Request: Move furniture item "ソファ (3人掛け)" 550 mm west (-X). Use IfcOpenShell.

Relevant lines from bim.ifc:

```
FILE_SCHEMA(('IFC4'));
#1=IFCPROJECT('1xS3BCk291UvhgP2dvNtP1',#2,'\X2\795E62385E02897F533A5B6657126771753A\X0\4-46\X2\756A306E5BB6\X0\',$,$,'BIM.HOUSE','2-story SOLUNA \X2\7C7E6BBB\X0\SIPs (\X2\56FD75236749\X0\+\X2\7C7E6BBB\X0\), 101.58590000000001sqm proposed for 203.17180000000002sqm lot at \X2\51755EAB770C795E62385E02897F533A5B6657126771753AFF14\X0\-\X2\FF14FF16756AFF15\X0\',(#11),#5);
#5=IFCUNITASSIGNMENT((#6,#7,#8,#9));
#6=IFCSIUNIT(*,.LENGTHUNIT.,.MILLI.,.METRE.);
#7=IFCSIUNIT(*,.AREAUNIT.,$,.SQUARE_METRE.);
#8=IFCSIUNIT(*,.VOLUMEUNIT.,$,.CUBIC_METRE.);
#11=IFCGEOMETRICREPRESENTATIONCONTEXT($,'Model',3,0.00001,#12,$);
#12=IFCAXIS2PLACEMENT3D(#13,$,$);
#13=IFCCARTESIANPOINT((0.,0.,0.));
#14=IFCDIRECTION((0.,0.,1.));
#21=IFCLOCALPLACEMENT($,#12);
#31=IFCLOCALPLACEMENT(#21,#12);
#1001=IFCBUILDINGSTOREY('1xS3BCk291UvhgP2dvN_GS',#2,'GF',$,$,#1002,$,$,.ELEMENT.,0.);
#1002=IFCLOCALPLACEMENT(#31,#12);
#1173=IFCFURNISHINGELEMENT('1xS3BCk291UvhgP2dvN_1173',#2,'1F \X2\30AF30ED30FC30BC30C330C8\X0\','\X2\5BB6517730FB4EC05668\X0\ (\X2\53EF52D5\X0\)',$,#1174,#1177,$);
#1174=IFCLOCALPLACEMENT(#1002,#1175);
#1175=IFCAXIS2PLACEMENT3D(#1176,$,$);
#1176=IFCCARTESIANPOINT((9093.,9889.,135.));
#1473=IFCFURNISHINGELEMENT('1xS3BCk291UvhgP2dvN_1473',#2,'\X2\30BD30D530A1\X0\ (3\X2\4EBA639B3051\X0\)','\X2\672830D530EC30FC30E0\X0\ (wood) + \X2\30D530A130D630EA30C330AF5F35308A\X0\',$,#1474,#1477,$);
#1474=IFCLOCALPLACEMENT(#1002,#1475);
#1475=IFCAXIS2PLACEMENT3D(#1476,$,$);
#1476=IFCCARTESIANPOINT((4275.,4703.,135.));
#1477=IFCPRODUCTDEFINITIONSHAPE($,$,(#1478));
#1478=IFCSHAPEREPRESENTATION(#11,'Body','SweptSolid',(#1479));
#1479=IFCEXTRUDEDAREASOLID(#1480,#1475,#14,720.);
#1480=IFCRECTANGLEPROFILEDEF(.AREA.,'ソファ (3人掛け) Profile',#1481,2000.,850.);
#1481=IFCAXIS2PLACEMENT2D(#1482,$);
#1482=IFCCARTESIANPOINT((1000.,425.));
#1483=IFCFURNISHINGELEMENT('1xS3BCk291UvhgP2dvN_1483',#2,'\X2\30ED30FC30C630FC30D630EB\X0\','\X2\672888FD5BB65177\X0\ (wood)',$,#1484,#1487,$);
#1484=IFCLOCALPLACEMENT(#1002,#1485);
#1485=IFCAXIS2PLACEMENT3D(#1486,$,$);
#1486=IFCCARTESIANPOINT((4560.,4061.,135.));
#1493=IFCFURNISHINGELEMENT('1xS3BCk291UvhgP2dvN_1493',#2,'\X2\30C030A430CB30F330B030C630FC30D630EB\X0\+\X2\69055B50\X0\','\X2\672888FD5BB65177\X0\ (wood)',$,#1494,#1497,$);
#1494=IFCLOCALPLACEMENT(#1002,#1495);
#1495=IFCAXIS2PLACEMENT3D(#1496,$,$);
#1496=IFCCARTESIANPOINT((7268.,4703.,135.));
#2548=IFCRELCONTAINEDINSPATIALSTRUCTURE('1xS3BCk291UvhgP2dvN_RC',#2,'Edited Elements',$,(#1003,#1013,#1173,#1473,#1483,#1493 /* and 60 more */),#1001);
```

```python
import ifcopenshell
import ifcopenshell.api.geometry
import ifcopenshell.util.placement
import ifcopenshell.util.unit

model = ifcopenshell.open("bim.ifc")
unit_scale = ifcopenshell.util.unit.calculate_unit_scale(model)

item = model.by_id(1473)
matrix = ifcopenshell.util.placement.get_local_placement(item.ObjectPlacement)
matrix[0, 3] -= 0.55 / unit_scale
ifcopenshell.api.geometry.edit_object_placement(model, product=item, matrix=matrix, is_si=False)

print(ifcopenshell.util.placement.get_local_placement(item.ObjectPlacement).round(3) + 0.0)

model.write("bim-out.ifc")
```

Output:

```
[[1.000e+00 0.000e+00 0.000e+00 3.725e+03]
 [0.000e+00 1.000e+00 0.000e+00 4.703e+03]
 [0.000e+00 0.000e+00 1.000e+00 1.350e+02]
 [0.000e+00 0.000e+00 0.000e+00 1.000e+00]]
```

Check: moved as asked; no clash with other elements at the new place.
